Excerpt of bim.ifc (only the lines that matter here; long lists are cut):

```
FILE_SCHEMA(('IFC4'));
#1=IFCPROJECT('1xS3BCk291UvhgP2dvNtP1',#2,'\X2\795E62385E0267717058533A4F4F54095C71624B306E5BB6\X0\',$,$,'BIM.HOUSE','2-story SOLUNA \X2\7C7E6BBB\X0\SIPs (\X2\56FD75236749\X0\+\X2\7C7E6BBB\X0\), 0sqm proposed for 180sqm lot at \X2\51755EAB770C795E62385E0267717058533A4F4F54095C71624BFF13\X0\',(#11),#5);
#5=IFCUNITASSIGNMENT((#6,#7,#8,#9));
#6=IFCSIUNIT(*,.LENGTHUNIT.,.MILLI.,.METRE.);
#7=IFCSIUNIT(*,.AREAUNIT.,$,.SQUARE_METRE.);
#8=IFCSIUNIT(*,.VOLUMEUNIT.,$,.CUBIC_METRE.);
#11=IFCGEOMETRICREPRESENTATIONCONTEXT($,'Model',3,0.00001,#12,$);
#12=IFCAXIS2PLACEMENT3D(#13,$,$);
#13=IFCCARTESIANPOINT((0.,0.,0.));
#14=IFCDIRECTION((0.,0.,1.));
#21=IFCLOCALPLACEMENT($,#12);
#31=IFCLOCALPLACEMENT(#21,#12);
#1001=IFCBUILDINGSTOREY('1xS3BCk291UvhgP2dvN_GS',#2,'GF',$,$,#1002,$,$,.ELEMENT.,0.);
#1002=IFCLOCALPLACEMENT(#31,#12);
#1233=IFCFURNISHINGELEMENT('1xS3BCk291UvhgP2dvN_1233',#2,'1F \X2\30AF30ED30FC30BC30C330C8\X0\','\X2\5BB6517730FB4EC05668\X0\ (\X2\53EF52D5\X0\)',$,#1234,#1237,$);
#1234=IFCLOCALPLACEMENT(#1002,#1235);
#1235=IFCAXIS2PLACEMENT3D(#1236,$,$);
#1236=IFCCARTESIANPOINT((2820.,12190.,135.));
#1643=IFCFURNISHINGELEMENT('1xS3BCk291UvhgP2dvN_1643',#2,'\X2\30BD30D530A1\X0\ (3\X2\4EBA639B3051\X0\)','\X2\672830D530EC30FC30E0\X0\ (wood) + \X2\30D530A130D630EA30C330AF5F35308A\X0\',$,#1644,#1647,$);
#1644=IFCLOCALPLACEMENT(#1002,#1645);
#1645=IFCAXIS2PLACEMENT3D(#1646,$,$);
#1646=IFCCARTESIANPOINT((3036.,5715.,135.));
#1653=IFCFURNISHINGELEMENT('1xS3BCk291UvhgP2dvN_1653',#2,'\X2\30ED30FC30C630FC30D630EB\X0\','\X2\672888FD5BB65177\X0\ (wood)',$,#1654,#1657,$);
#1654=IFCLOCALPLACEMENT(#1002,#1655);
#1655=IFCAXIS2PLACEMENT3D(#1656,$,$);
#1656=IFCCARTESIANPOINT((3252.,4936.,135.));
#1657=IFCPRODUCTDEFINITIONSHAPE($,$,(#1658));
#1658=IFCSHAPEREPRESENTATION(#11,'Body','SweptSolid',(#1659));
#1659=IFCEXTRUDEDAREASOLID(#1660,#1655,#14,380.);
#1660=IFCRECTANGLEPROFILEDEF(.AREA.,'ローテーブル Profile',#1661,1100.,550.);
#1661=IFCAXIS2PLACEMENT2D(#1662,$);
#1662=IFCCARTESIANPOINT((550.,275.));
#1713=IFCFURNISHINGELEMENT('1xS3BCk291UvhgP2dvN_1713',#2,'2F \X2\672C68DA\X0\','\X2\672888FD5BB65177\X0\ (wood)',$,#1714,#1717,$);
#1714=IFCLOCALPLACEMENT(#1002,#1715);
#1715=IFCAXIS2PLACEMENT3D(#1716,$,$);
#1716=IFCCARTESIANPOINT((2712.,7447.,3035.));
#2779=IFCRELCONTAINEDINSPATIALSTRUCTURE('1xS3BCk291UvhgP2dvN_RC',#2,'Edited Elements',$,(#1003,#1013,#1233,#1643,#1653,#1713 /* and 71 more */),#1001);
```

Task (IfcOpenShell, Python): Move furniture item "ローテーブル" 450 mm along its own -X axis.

```python
import ifcopenshell
import ifcopenshell.api.geometry
import ifcopenshell.util.placement

model = ifcopenshell.open("bim.ifc")

item = model.by_guid("1xS3BCk291UvhgP2dvN_1653")
matrix = ifcopenshell.util.placement.get_local_placement(item.ObjectPlacement)
matrix[:3, 3] -= matrix[:3, 0] * 450.0
ifcopenshell.api.geometry.edit_object_placement(model, product=item, matrix=matrix, is_si=False)

print(ifcopenshell.util.placement.get_local_placement(item.ObjectPlacement).round(3) + 0.0)

model.write("bim_updated.ifc")
```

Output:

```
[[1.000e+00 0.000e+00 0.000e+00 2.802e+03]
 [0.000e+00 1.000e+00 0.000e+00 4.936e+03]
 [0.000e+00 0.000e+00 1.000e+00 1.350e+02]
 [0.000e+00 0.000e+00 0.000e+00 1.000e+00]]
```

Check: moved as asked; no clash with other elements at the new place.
